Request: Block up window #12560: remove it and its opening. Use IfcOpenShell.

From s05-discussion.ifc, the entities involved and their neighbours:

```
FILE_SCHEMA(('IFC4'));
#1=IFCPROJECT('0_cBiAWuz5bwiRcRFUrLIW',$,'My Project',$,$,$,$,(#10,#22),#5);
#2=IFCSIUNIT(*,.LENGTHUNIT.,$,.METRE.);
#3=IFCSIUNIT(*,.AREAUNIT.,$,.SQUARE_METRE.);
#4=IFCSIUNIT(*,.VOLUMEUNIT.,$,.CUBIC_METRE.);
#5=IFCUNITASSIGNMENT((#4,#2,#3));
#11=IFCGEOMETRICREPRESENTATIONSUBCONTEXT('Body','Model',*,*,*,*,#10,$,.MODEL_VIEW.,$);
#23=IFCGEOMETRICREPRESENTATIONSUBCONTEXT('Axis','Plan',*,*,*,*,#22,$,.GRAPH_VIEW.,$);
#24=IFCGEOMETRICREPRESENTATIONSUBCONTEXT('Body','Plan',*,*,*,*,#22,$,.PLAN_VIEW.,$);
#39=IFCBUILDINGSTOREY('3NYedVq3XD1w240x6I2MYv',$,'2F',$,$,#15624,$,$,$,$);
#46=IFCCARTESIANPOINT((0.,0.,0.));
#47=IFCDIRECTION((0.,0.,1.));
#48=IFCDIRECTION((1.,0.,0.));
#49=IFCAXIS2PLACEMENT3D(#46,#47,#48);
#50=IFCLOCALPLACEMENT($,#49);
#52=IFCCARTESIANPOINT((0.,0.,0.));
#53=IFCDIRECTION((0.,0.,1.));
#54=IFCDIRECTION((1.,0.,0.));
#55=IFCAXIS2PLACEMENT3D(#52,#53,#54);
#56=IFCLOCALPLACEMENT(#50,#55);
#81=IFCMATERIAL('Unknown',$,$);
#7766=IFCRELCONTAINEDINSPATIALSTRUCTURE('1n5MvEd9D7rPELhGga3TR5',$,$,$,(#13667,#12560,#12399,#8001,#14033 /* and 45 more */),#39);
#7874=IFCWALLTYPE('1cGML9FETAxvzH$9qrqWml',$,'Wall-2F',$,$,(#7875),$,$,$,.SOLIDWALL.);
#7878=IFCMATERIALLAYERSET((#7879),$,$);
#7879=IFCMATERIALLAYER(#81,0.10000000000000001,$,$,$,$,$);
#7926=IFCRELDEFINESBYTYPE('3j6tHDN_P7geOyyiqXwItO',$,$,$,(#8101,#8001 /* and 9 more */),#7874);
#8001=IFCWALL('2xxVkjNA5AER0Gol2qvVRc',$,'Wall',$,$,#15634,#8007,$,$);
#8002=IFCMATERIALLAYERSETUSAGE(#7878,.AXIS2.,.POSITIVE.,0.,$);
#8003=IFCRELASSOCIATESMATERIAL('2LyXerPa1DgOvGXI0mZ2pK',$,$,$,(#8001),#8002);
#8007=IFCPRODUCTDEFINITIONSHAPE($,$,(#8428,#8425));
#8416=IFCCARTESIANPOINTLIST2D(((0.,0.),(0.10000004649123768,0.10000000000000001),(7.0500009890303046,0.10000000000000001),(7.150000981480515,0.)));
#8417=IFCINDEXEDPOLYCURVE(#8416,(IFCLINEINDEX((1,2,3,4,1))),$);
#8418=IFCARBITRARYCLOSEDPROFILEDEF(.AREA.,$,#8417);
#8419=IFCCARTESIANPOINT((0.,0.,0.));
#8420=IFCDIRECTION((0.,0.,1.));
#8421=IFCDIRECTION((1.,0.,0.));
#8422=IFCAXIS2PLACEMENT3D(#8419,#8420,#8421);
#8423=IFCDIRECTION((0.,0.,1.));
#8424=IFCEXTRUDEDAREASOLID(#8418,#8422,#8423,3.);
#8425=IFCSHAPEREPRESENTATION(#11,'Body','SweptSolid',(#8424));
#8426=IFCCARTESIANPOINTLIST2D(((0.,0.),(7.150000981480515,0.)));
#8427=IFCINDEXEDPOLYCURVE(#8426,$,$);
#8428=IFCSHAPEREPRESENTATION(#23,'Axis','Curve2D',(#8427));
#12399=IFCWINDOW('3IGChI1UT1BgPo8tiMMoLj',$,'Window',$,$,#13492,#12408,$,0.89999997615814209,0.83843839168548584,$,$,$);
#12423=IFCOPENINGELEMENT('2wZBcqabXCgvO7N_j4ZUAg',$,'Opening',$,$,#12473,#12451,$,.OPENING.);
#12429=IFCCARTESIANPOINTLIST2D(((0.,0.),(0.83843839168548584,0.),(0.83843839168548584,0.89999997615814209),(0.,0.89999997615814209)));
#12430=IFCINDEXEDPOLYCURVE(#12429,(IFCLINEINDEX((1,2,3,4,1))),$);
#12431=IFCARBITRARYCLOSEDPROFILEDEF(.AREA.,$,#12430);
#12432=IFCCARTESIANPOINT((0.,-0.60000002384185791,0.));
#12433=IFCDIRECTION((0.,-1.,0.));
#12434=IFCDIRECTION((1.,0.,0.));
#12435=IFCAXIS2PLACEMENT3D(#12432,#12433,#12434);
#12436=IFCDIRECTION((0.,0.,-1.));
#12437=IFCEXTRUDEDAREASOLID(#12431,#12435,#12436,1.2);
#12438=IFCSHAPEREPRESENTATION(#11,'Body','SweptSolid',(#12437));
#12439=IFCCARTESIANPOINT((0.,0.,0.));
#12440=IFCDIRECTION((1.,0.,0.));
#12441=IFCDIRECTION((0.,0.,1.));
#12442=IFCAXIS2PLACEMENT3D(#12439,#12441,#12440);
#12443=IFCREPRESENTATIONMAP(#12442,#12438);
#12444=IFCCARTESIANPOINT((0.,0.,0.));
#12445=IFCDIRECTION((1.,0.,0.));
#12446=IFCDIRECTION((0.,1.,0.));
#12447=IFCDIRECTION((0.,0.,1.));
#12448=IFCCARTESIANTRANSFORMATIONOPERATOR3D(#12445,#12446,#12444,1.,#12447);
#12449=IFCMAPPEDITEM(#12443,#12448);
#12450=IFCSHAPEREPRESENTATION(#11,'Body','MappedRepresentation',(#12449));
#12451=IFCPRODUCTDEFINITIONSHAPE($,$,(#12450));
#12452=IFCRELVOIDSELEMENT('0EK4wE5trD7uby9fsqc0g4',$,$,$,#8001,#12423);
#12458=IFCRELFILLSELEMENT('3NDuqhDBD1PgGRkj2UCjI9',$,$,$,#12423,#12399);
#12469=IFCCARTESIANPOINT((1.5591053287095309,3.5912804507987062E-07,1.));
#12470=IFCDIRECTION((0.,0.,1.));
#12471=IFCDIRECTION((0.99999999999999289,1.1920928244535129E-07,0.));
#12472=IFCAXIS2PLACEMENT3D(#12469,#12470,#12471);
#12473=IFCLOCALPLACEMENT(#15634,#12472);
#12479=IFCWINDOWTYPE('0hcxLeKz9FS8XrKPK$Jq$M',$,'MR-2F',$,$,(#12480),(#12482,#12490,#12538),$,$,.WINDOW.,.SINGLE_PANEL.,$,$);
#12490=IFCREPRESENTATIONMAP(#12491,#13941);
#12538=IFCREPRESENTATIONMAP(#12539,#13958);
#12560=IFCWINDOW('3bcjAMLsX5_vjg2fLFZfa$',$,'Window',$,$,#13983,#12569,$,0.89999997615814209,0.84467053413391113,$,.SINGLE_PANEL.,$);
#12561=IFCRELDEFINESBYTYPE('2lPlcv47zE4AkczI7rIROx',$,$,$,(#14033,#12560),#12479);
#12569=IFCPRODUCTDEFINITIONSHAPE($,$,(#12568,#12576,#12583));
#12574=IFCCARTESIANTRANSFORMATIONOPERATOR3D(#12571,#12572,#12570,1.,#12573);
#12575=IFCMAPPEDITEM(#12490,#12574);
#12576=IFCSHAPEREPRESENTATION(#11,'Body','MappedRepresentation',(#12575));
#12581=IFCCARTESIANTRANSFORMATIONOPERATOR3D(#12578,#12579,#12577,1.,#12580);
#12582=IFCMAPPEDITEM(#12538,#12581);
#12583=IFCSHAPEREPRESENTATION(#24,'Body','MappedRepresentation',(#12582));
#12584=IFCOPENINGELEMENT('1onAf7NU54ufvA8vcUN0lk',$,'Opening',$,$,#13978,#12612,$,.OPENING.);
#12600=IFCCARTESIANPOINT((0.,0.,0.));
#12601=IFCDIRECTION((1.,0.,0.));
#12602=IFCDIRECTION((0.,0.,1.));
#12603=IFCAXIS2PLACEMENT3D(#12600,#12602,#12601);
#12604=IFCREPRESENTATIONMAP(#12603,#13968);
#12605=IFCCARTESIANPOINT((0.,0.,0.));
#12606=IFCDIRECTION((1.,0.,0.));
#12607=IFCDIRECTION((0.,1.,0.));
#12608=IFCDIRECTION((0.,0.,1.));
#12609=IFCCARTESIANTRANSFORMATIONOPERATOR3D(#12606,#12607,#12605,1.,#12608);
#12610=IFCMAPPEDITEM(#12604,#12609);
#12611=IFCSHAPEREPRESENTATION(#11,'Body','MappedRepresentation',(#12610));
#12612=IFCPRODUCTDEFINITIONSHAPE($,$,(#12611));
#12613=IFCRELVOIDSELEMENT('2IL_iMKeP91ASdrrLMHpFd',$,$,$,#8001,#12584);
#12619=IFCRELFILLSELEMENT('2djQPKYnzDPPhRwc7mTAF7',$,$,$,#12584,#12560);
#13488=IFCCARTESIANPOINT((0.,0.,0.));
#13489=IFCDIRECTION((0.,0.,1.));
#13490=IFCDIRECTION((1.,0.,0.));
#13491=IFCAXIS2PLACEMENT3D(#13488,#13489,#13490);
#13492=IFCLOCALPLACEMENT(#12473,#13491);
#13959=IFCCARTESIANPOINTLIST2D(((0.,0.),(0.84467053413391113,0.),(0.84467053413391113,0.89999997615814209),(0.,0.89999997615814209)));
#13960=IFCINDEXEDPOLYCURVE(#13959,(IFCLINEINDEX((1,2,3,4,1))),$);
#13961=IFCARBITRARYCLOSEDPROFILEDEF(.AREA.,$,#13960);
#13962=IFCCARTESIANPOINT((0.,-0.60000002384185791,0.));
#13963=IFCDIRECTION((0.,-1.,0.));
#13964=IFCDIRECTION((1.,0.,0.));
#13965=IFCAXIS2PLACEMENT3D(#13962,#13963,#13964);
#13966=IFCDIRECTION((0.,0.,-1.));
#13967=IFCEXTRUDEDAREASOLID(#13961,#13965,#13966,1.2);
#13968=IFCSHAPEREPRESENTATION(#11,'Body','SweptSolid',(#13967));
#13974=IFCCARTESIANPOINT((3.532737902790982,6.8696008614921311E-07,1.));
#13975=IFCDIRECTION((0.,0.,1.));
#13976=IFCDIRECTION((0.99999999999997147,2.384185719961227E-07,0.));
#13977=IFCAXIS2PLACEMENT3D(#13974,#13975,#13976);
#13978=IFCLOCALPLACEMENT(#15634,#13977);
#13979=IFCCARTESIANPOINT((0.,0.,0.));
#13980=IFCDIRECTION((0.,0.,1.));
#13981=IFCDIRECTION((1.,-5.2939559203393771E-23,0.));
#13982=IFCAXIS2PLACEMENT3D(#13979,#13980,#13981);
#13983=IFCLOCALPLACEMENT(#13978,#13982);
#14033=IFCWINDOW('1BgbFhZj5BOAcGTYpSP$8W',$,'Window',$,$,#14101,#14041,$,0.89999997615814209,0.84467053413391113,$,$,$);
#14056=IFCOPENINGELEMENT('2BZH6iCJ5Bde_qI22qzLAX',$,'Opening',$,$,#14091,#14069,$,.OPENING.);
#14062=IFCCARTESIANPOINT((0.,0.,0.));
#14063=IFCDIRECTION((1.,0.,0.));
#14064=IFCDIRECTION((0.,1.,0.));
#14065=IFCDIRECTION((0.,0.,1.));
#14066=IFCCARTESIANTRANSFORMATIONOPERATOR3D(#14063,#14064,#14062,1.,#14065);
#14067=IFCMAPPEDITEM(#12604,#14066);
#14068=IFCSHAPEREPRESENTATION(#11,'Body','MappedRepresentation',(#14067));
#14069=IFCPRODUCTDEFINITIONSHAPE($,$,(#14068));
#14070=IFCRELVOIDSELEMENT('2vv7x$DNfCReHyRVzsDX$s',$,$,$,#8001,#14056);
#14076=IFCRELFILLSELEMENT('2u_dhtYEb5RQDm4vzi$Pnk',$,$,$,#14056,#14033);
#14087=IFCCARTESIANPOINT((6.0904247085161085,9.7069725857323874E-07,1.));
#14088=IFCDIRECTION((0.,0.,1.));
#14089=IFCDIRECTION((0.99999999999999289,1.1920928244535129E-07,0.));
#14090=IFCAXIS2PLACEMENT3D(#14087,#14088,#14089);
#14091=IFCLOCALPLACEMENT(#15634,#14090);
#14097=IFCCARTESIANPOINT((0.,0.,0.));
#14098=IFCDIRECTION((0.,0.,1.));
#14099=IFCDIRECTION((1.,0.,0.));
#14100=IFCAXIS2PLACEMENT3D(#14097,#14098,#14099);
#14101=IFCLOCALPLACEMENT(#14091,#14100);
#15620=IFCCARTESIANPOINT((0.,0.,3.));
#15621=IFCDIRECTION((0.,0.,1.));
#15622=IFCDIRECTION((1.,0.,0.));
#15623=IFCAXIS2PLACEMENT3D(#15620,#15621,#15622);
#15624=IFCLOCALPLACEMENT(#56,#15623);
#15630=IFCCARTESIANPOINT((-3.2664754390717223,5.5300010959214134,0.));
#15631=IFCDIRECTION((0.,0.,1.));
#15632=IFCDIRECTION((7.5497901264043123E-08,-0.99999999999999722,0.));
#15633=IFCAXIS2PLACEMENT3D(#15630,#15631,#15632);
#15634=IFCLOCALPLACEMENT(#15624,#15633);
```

```python
import ifcopenshell
import ifcopenshell.api.feature
import ifcopenshell.api.root
import ifcopenshell.geom
import ifcopenshell.util.shape

model = ifcopenshell.open("s05-discussion.ifc")
settings = ifcopenshell.geom.settings()


def volume(element):
    """Net volume in cubic metres, openings subtracted."""
    shape = ifcopenshell.geom.create_shape(settings, element)
    return ifcopenshell.util.shape.get_volume(shape.geometry)


window = model.by_guid("3bcjAMLsX5_vjg2fLFZfa$")
opening = window.FillsVoids[0].RelatingOpeningElement
wall = opening.VoidsElements[0].RelatingBuildingElement
before = volume(wall)

ifcopenshell.api.root.remove_product(model, product=window)
ifcopenshell.api.feature.remove_feature(model, feature=opening)

after = volume(wall)

print(f"wall volume {before:.3f} -> {after:.3f} m3")

model.write("s05-discussion-out.ifc")
```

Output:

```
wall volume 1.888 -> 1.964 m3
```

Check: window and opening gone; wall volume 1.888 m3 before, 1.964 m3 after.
